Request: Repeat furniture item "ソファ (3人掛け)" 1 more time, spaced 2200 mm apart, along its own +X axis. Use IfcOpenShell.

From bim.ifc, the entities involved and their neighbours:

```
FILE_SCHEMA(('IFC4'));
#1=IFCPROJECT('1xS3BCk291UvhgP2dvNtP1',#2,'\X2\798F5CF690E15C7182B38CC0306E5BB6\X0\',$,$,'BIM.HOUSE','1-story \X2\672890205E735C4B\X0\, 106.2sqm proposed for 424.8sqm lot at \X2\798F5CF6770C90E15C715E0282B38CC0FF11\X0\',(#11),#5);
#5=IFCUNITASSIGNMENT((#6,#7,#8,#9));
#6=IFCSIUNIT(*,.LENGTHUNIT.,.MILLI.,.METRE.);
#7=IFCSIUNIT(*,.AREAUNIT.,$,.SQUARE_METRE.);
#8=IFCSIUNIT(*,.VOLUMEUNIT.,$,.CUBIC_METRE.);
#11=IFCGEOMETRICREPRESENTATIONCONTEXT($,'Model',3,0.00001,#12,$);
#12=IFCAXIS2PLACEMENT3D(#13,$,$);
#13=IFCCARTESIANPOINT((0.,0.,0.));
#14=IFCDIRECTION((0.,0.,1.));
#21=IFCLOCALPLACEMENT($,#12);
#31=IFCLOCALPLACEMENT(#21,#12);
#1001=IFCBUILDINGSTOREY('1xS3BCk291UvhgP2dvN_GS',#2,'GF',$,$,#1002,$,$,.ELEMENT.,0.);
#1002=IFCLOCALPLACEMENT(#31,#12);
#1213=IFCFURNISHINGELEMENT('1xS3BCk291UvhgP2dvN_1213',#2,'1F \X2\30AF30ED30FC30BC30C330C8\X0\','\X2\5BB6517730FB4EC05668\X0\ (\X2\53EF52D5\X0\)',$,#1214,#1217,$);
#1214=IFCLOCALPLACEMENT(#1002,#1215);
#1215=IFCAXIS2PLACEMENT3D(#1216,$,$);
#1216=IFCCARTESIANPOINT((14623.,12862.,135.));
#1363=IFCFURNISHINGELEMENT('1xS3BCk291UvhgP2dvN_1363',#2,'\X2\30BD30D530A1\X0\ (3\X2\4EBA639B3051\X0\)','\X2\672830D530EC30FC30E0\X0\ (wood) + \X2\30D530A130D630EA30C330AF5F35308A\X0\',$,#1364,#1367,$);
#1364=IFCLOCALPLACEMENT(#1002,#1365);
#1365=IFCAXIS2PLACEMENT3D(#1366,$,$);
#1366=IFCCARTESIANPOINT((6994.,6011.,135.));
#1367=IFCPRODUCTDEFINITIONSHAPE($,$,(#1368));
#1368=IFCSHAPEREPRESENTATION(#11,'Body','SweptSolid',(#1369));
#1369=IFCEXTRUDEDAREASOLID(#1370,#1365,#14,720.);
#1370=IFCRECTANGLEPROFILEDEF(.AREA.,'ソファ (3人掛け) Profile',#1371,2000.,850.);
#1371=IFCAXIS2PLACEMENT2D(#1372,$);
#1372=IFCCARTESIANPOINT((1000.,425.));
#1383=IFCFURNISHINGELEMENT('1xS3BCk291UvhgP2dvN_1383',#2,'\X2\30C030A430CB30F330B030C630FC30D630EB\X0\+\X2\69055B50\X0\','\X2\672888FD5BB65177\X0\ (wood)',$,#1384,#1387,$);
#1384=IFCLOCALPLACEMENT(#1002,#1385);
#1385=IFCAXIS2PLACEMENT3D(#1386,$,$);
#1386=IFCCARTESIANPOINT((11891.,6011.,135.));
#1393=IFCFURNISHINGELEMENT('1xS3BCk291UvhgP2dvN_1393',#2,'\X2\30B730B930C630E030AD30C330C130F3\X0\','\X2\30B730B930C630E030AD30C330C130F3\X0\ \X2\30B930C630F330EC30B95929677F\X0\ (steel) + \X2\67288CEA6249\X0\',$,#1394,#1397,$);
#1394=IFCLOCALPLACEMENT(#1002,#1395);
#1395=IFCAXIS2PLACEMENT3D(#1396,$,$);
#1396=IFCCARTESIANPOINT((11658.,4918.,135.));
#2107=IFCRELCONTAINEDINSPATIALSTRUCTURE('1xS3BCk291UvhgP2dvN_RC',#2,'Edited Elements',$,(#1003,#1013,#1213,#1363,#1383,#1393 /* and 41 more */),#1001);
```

```python
import ifcopenshell
import ifcopenshell.api.geometry
import ifcopenshell.api.root
import ifcopenshell.util.element
import ifcopenshell.util.placement
import ifcopenshell.util.unit

model = ifcopenshell.open("bim.ifc")
unit_scale = ifcopenshell.util.unit.calculate_unit_scale(model)


def reuse_history(source, copy):
    """copy_class also copies each property set's owner history, people and application; keep the originals."""
    for rel in copy.IsDefinedBy:
        if rel.is_a("IfcRelDefinesByProperties") and (history := rel.RelatingPropertyDefinition.OwnerHistory):
            rel.RelatingPropertyDefinition.OwnerHistory = source.OwnerHistory
            ifcopenshell.util.element.remove_deep2(model, history)


source = model.by_id(1363)
base = ifcopenshell.util.placement.get_local_placement(source.ObjectPlacement)
step = base[:3, 0] * 2.2 / unit_scale

for i in range(1, 2):
    copy = ifcopenshell.api.root.copy_class(model, product=source)
    copy.Representation = ifcopenshell.util.element.copy_deep(
        model, source.Representation, exclude=["IfcGeometricRepresentationContext", "IfcRepresentationMap"]
    )
    reuse_history(source, copy)
    matrix = base.copy()
    matrix[:3, 3] += i * step
    print("added at", matrix[:3, 3].round(3) + 0.0)
    ifcopenshell.api.geometry.edit_object_placement(model, product=copy, matrix=matrix, is_si=False)

model.write("bim_updated.ifc")
```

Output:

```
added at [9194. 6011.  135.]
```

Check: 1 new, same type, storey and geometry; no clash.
